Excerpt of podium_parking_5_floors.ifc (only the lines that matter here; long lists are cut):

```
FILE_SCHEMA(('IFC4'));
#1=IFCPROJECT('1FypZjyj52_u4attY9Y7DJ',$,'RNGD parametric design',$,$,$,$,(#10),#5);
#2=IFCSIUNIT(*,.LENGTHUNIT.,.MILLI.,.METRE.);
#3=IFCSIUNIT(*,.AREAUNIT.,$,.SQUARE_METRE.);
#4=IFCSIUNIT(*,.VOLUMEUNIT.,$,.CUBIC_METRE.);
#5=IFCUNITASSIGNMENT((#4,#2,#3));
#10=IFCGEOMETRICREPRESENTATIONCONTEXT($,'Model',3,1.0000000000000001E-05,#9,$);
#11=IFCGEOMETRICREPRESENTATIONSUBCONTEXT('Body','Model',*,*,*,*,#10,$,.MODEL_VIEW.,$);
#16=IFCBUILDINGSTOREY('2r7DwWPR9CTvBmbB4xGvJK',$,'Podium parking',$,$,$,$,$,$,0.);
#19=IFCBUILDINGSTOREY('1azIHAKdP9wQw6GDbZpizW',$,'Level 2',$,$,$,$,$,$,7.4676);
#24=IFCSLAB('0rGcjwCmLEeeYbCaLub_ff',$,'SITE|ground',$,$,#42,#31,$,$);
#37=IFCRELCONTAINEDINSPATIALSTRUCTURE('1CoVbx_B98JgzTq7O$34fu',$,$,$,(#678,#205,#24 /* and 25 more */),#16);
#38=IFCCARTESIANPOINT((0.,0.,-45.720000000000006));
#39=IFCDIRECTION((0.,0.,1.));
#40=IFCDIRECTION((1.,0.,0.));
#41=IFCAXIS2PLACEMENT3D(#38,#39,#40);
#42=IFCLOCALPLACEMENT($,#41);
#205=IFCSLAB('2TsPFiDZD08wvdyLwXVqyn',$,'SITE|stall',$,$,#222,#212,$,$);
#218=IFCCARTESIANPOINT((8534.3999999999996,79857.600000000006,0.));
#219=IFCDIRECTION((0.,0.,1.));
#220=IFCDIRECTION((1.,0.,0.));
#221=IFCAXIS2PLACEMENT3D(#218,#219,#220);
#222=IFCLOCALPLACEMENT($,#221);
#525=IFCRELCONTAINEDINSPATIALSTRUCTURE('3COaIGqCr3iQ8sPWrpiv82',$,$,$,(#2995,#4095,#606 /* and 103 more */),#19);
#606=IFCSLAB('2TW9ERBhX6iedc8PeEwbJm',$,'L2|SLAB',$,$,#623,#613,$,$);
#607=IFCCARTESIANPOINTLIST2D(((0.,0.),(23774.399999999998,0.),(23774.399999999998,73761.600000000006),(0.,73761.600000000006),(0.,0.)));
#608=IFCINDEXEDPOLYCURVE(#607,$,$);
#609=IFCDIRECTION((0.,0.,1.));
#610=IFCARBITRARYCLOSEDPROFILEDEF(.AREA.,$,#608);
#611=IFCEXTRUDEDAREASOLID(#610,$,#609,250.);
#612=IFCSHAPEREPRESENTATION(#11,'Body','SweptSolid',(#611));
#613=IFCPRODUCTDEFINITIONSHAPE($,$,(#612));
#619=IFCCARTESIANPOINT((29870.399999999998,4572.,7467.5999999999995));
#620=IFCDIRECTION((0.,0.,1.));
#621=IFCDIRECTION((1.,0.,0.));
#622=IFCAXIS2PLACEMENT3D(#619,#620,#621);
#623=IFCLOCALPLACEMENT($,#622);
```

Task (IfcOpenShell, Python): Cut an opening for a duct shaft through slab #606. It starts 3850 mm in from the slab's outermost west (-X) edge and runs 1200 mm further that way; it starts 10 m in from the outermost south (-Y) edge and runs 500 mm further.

```python
import numpy as np
import ifcopenshell
import ifcopenshell.api.feature
import ifcopenshell.api.geometry
import ifcopenshell.api.root
import ifcopenshell.geom
import ifcopenshell.util.placement
import ifcopenshell.util.representation
import ifcopenshell.util.shape
import ifcopenshell.util.unit

model = ifcopenshell.open("podium_parking_5_floors.ifc")
unit_scale = ifcopenshell.util.unit.calculate_unit_scale(model)
settings = ifcopenshell.geom.settings()


def volume(element):
    """Net volume in cubic metres, openings subtracted."""
    shape = ifcopenshell.geom.create_shape(settings, element)
    return ifcopenshell.util.shape.get_volume(shape.geometry)


slab = model.by_guid("2TW9ERBhX6iedc8PeEwbJm")
before = volume(slab)

# Extent in the slab's own axes, in metres. The edges named are its -X and -Y sides.
slab_shape = ifcopenshell.geom.create_shape(settings, slab)
vertices = ifcopenshell.util.shape.get_vertices(slab_shape.geometry)
x_min, y_min, bottom = vertices.min(axis=0)
top = vertices[:, 2].max()

opening = ifcopenshell.api.root.create_entity(model, ifc_class="IfcOpeningElement", name="Duct shaft opening", predefined_type="OPENING")
context = ifcopenshell.util.representation.get_context(model, "Model", "Body", "MODEL_VIEW")
width, depth = 1.2, 0.5
outline = [(0.0, 0.0), (width, 0.0), (width, depth), (0.0, depth), (0.0, 0.0)]
# Overshoot both faces by 50 mm so the cut is clean.
shape = ifcopenshell.api.geometry.add_slab_representation(
    model, context=context, depth=top - bottom + 0.1, polyline=outline
)
ifcopenshell.api.geometry.assign_representation(model, product=opening, representation=shape)

matrix = ifcopenshell.util.placement.get_local_placement(slab.ObjectPlacement)
matrix[:, 3] = matrix @ np.append(np.array([x_min + 3.85, y_min + 10, bottom - 0.05]) / unit_scale, 1.0)
ifcopenshell.api.geometry.edit_object_placement(model, product=opening, matrix=matrix, is_si=False)
ifcopenshell.api.feature.add_feature(model, feature=opening, element=slab)

after = volume(slab)

print(f"slab volume {before:.3f} -> {after:.3f} m3")

model.write("podium_parking_5_floors_v2.ifc")
```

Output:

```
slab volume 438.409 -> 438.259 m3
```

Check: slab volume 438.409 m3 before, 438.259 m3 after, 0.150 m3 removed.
